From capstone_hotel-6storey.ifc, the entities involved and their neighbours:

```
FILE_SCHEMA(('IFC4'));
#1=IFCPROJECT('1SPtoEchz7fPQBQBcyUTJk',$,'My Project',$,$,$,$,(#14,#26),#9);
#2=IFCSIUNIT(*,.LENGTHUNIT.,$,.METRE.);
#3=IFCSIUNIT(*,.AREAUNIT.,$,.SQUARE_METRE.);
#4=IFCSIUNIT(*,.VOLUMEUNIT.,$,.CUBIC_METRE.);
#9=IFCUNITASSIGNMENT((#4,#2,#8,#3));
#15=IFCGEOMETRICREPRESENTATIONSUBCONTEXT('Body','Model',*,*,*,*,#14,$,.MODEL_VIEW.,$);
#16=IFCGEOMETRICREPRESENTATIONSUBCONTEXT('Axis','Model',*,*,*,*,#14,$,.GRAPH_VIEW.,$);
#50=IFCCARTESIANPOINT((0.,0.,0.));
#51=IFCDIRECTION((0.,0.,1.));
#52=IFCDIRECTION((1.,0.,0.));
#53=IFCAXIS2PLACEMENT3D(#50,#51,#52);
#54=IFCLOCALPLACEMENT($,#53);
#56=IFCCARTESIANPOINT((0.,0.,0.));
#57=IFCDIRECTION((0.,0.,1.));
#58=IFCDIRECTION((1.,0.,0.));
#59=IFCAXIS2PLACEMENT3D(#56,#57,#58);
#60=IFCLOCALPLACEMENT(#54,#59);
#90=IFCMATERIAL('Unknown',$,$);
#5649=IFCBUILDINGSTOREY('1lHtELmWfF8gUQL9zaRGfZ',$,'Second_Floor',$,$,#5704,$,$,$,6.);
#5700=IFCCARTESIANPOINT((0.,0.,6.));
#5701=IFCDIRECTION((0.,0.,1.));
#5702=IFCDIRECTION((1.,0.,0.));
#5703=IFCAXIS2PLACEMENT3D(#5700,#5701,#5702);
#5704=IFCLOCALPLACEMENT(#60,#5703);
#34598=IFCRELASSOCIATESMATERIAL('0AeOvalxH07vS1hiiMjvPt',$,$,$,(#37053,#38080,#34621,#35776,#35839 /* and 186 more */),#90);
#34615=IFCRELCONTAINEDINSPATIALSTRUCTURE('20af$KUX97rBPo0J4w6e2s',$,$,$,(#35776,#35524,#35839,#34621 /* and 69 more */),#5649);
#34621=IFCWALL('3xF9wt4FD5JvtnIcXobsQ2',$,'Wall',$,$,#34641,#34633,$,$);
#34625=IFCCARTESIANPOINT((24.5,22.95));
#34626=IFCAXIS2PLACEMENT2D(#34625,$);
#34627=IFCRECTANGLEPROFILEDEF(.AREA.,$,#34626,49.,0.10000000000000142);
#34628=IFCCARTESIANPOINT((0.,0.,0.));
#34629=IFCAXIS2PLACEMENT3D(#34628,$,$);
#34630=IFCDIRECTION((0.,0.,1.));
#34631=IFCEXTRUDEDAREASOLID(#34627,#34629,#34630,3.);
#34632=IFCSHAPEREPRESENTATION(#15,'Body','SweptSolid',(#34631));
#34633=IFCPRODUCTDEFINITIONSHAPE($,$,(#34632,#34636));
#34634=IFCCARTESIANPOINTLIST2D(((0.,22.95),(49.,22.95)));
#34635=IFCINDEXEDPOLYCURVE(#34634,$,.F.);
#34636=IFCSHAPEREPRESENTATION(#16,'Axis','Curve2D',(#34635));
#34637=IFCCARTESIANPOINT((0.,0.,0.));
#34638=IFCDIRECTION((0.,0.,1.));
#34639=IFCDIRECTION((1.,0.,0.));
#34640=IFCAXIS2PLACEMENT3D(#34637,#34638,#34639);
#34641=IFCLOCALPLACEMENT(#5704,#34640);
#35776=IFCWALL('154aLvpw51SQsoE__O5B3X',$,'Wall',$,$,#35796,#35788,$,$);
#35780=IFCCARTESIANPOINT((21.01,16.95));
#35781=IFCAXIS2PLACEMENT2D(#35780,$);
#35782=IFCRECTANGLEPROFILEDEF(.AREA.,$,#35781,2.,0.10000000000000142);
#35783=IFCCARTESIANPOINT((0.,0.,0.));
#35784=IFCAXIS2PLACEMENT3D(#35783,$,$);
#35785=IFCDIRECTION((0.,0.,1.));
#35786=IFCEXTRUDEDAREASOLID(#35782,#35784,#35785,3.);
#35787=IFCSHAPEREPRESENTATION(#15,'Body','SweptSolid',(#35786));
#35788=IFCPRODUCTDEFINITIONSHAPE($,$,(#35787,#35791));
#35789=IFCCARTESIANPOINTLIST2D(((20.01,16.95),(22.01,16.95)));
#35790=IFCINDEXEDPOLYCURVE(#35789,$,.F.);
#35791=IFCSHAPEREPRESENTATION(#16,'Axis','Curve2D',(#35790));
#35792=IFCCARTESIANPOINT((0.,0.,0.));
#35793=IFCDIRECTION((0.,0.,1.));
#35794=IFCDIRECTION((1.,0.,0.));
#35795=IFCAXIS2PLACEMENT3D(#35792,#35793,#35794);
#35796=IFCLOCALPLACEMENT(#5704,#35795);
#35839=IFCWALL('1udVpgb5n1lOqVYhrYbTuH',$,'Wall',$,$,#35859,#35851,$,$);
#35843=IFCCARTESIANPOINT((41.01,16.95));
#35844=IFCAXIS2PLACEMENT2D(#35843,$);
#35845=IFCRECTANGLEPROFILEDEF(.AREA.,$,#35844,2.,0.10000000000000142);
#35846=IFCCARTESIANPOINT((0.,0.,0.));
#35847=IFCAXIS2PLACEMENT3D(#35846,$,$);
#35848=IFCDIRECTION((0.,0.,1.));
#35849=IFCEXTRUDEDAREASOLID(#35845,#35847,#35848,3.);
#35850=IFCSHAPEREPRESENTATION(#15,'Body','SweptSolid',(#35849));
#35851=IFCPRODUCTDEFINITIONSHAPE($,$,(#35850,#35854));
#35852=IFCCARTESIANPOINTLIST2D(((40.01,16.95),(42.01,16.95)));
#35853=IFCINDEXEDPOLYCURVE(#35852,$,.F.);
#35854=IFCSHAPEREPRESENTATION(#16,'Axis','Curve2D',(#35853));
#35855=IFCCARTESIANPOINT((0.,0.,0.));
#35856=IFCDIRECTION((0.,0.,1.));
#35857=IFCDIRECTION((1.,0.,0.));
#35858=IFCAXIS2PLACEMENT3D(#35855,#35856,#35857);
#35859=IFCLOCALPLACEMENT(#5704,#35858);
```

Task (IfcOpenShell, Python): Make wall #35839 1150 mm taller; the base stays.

```python
import ifcopenshell
import ifcopenshell.geom
import ifcopenshell.util.representation
import ifcopenshell.util.shape

model = ifcopenshell.open("capstone_hotel-6storey.ifc")
settings = ifcopenshell.geom.settings()


def volume(element):
    """Net volume in cubic metres, openings subtracted."""
    shape = ifcopenshell.geom.create_shape(settings, element)
    return ifcopenshell.util.shape.get_volume(shape.geometry)


wall = model.by_guid("1udVpgb5n1lOqVYhrYbTuH")
before = volume(wall)

body = ifcopenshell.util.representation.get_representation(wall, "Model", "Body")
solid = body.Items[0]
old_height = solid.Depth
solid.Depth += 1.15
after = volume(wall)

print(f"height {old_height:g} -> {solid.Depth:g}, volume {before:.3f} -> {after:.3f} m3")

model.write("capstone_hotel-6storey_updated.ifc")
```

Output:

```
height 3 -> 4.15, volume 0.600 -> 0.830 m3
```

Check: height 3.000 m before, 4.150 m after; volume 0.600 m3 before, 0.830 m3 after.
